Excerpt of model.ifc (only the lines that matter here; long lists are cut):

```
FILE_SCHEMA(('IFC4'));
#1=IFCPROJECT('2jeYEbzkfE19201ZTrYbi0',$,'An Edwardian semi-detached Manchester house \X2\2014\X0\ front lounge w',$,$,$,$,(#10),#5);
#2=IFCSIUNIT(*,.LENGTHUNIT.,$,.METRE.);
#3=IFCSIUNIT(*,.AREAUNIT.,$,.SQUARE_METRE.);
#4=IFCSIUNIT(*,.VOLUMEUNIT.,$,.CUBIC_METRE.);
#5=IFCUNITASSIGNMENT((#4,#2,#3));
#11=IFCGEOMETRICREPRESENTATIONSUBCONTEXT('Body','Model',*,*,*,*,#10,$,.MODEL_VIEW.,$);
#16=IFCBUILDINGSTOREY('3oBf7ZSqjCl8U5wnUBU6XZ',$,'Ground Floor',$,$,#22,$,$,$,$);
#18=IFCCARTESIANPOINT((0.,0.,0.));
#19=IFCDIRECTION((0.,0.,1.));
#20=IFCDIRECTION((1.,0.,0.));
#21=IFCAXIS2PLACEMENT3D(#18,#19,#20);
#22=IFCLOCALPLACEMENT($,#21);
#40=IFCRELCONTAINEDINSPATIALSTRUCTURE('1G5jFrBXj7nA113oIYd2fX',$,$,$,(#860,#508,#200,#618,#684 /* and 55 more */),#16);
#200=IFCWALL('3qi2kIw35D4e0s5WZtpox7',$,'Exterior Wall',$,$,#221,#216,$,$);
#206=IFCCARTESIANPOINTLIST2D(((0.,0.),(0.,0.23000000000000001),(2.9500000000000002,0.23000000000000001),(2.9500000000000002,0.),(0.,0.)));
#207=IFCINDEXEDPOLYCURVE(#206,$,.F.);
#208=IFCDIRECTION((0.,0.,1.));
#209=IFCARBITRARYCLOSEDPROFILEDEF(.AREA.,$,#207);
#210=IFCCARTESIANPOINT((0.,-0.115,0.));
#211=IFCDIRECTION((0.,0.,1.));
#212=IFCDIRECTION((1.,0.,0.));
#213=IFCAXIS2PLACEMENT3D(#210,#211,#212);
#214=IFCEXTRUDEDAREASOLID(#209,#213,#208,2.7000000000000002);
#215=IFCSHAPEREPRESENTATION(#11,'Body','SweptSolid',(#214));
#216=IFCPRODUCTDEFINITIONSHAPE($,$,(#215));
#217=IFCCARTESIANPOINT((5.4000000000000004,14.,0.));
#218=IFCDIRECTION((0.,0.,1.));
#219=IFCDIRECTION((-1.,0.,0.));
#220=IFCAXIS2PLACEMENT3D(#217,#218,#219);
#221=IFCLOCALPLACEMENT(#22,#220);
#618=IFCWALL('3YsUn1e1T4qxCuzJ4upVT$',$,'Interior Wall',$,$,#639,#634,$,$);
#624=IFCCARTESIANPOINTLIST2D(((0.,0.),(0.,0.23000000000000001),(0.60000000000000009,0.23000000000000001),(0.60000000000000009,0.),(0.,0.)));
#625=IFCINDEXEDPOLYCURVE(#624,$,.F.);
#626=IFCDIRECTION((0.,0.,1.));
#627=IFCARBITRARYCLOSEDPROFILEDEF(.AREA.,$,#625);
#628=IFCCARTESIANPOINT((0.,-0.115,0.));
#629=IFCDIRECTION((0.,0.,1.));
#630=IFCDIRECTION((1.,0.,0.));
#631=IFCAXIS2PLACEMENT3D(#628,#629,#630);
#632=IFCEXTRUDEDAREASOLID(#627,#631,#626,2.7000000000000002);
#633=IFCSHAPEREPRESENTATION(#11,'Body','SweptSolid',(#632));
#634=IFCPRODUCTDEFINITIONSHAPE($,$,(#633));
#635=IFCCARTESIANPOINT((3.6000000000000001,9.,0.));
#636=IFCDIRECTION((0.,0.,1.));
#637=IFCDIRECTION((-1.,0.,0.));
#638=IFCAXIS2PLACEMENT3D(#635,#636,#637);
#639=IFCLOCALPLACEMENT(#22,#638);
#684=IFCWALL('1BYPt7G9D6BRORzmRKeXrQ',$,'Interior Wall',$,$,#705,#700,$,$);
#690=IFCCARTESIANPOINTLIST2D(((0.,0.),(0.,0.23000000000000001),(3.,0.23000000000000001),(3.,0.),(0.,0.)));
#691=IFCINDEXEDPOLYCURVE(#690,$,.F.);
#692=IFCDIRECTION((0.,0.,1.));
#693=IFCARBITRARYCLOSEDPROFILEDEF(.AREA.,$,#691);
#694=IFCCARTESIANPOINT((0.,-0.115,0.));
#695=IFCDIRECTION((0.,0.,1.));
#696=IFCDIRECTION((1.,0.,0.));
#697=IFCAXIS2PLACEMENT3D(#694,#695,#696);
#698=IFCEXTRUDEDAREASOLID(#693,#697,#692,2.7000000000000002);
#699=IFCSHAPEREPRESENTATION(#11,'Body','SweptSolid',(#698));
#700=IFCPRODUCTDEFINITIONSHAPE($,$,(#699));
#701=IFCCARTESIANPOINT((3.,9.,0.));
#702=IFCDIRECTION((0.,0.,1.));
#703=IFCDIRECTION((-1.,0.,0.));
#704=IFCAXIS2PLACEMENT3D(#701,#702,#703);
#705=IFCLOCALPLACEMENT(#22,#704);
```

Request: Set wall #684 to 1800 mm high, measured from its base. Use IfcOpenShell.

```python
import ifcopenshell
import ifcopenshell.geom
import ifcopenshell.util.representation
import ifcopenshell.util.shape

model = ifcopenshell.open("model.ifc")
settings = ifcopenshell.geom.settings()


def volume(element):
    """Net volume in cubic metres, openings subtracted."""
    shape = ifcopenshell.geom.create_shape(settings, element)
    return ifcopenshell.util.shape.get_volume(shape.geometry)


wall = model.by_id(684)
before = volume(wall)

body = ifcopenshell.util.representation.get_representation(wall, "Model", "Body")
solid = body.Items[0]
old_height = solid.Depth
solid.Depth = 1.8
after = volume(wall)

print(f"height {old_height:g} -> {solid.Depth:g}, volume {before:.3f} -> {after:.3f} m3")

model.write("model_rev.ifc")
```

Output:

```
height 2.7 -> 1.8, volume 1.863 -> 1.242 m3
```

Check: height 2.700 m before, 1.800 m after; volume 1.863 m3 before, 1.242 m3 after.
